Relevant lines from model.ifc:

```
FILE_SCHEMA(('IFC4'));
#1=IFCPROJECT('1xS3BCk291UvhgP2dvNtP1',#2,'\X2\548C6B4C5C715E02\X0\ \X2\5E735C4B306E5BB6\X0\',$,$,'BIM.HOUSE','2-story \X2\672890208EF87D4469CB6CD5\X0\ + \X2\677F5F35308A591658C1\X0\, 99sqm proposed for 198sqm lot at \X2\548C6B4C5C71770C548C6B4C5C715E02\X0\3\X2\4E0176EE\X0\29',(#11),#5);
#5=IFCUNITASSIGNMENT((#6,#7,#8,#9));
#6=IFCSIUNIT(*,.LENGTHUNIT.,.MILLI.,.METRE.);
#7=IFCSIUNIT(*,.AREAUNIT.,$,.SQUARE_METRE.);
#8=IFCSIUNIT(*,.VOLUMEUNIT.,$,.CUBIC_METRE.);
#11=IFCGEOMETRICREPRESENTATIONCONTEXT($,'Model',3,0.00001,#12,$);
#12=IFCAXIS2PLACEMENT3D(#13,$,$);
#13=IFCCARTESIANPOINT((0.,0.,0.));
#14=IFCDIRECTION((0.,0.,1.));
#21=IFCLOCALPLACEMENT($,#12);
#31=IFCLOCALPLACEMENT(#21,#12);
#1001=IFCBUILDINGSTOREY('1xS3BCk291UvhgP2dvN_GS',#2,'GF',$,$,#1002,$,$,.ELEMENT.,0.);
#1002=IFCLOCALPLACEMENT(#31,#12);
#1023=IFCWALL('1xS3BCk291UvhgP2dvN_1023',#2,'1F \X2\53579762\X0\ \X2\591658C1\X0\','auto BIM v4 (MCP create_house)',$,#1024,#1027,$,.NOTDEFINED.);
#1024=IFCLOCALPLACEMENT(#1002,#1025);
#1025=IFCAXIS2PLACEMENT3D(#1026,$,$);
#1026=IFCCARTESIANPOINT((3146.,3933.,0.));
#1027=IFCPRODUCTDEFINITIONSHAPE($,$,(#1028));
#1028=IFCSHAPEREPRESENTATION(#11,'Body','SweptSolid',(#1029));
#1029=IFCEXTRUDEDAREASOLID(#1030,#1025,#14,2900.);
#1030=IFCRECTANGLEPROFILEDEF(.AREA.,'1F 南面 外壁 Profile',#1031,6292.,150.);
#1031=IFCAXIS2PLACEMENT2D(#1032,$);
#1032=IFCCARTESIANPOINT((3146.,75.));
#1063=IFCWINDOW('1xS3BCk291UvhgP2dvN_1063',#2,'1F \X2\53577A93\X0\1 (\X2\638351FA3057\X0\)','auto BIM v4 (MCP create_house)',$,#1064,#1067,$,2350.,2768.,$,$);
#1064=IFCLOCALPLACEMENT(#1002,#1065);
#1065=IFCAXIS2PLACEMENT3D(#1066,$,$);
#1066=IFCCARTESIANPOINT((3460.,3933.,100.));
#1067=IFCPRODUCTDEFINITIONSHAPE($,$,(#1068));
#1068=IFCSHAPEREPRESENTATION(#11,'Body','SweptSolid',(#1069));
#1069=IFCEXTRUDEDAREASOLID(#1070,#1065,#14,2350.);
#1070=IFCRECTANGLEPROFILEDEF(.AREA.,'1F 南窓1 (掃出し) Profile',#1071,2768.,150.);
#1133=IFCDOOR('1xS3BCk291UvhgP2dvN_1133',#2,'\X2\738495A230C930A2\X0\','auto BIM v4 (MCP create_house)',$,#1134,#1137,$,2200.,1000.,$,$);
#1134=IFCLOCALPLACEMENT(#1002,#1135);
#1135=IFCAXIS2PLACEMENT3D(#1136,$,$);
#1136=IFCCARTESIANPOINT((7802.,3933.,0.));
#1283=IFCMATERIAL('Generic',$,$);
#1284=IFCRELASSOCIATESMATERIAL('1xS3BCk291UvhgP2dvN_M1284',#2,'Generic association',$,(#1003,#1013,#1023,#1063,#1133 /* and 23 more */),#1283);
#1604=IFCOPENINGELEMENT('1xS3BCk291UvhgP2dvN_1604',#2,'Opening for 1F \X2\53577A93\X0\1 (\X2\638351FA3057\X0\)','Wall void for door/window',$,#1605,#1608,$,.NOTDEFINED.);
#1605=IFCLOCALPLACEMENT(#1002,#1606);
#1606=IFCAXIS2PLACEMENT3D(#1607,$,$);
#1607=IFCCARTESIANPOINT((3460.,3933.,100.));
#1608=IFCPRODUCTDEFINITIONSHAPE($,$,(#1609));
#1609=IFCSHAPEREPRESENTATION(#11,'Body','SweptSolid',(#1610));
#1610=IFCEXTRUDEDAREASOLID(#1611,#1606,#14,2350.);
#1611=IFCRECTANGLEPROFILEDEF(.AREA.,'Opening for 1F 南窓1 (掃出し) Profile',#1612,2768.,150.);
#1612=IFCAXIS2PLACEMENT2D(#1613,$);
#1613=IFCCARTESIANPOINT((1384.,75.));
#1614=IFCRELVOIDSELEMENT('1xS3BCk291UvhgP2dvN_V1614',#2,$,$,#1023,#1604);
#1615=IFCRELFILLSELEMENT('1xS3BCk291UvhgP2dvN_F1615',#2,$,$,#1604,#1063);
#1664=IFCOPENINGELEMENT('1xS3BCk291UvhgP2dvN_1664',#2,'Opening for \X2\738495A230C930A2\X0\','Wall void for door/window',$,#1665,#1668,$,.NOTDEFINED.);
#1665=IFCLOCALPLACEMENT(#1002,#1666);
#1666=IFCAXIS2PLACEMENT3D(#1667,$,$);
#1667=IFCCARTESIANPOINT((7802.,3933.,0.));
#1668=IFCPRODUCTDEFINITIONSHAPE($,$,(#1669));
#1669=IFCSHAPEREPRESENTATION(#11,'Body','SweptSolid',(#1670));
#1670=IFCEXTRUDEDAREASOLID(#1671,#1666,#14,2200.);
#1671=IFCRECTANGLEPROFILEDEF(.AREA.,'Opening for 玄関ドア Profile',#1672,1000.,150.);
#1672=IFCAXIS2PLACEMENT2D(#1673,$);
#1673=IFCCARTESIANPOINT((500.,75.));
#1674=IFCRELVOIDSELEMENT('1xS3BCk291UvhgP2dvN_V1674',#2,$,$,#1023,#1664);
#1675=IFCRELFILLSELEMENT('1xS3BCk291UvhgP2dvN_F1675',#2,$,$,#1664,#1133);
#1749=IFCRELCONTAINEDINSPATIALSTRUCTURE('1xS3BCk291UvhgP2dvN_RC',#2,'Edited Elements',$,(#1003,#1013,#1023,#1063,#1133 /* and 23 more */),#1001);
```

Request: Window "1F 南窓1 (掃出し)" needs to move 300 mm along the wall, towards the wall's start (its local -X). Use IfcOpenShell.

```python
import ifcopenshell
import ifcopenshell.api.geometry
import ifcopenshell.util.placement
import ifcopenshell.util.unit

model = ifcopenshell.open("model.ifc")
unit_scale = ifcopenshell.util.unit.calculate_unit_scale(model)

window = model.by_guid("1xS3BCk291UvhgP2dvN_1063")
opening = window.FillsVoids[0].RelatingOpeningElement
wall = opening.VoidsElements[0].RelatingBuildingElement

wall_matrix = ifcopenshell.util.placement.get_local_placement(wall.ObjectPlacement)
shift = wall_matrix[:3, 0] * -0.3 / unit_scale
before = ifcopenshell.util.placement.get_local_placement(window.ObjectPlacement)[:3, 3].copy()

# The window is not placed relative to its opening, so move both.
for product in (opening, window):
    matrix = ifcopenshell.util.placement.get_local_placement(product.ObjectPlacement)
    matrix[:3, 3] += shift
    ifcopenshell.api.geometry.edit_object_placement(model, product=product, matrix=matrix, is_si=False)

after = ifcopenshell.util.placement.get_local_placement(window.ObjectPlacement)[:3, 3]
print("window moved by", (after - before).round(3) + 0.0)

model.write("model_v2.ifc")
```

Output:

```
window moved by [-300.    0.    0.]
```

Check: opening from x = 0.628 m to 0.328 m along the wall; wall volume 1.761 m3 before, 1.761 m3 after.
